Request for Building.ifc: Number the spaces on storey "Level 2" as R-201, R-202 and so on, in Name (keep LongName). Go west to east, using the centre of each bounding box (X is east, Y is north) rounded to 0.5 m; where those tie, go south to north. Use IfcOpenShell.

First a look at what the model holds.

```python
import ifcopenshell
import ifcopenshell.util.element
import ifcopenshell.util.placement

model = ifcopenshell.open("Building.ifc")
print(model.schema)
storey = next(s for s in model.by_type("IfcBuildingStorey") if s.Name == "Level 2")
spaces = [e for e in ifcopenshell.util.element.get_decomposition(storey) if e.is_a("IfcSpace")]
for e in sorted(spaces, key=lambda e: e.id()):
    origin = ifcopenshell.util.placement.get_local_placement(e.ObjectPlacement)[:3, 3]
    print(e.id(), e.Name, e.LongName, origin.round(2) + 0.0, sep=" | ")
```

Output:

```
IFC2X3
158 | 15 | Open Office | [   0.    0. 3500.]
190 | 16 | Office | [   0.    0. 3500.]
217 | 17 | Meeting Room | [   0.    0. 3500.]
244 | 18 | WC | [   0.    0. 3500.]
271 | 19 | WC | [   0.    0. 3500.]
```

```python
import ifcopenshell
import ifcopenshell.geom
import ifcopenshell.util.element
import ifcopenshell.util.shape

model = ifcopenshell.open("Building.ifc")
settings = ifcopenshell.geom.settings()
settings.set("use-world-coords", True)


def centre(element):
    shape = ifcopenshell.geom.create_shape(settings, element)
    return ifcopenshell.util.shape.get_bbox_centroid(shape.geometry)


storey = next(s for s in model.by_type("IfcBuildingStorey") if s.Name == "Level 2")
spaces = [e for e in ifcopenshell.util.element.get_decomposition(storey) if e.is_a("IfcSpace")]

# Insertion points can sit at a corner or the storey origin, so sort by the geometry (in metres).
centres = {e: centre(e) for e in spaces}
spaces.sort(key=lambda e: (round(centres[e][0] / 0.5), centres[e][1]))

for i, e in enumerate(spaces, start=1):
    number = f"R-2{i:02d}"
    e.Name = number
    print(e.id(), number)

model.write("Building_rev.ifc")
```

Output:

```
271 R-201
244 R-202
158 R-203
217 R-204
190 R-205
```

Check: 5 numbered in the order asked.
